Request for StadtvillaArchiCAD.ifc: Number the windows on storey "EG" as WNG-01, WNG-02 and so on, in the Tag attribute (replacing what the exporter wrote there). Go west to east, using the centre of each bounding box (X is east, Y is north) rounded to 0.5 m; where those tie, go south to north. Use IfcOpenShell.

First a look at what the model holds.

```python
import ifcopenshell
import ifcopenshell.util.element
import ifcopenshell.util.placement

model = ifcopenshell.open("StadtvillaArchiCAD.ifc")
print(model.schema)
storey = next(s for s in model.by_type("IfcBuildingStorey") if s.Name == "EG")
windows = [e for e in ifcopenshell.util.element.get_decomposition(storey) if e.is_a("IfcWindow")]
for e in sorted(windows, key=lambda e: e.id()):
    origin = ifcopenshell.util.placement.get_local_placement(e.ObjectPlacement)[:3, 3]
    print(e.id(), e.Tag, e.Name, origin.round(2) + 0.0, sep=" | ")
```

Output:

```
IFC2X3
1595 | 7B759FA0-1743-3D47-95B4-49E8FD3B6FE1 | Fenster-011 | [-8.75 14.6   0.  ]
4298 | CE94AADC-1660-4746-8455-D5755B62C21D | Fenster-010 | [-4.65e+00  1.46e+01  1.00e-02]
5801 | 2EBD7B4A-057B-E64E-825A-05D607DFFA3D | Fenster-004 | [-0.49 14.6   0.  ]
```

```python
import ifcopenshell
import ifcopenshell.geom
import ifcopenshell.util.element
import ifcopenshell.util.shape

model = ifcopenshell.open("StadtvillaArchiCAD.ifc")
settings = ifcopenshell.geom.settings()
settings.set("use-world-coords", True)


def centre(element):
    shape = ifcopenshell.geom.create_shape(settings, element)
    return ifcopenshell.util.shape.get_bbox_centroid(shape.geometry)


storey = next(s for s in model.by_type("IfcBuildingStorey") if s.Name == "EG")
windows = [e for e in ifcopenshell.util.element.get_decomposition(storey) if e.is_a("IfcWindow")]

# Insertion points can sit at a corner or the storey origin, so sort by the geometry (in metres).
centres = {e: centre(e) for e in windows}
windows.sort(key=lambda e: (round(centres[e][0] / 0.5), centres[e][1]))

for i, e in enumerate(windows, start=1):
    number = f"WNG-{i:02d}"
    e.Tag = number
    print(e.id(), number)

model.write("StadtvillaArchiCAD-out.ifc")
```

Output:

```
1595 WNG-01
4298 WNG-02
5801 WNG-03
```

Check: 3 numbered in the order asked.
